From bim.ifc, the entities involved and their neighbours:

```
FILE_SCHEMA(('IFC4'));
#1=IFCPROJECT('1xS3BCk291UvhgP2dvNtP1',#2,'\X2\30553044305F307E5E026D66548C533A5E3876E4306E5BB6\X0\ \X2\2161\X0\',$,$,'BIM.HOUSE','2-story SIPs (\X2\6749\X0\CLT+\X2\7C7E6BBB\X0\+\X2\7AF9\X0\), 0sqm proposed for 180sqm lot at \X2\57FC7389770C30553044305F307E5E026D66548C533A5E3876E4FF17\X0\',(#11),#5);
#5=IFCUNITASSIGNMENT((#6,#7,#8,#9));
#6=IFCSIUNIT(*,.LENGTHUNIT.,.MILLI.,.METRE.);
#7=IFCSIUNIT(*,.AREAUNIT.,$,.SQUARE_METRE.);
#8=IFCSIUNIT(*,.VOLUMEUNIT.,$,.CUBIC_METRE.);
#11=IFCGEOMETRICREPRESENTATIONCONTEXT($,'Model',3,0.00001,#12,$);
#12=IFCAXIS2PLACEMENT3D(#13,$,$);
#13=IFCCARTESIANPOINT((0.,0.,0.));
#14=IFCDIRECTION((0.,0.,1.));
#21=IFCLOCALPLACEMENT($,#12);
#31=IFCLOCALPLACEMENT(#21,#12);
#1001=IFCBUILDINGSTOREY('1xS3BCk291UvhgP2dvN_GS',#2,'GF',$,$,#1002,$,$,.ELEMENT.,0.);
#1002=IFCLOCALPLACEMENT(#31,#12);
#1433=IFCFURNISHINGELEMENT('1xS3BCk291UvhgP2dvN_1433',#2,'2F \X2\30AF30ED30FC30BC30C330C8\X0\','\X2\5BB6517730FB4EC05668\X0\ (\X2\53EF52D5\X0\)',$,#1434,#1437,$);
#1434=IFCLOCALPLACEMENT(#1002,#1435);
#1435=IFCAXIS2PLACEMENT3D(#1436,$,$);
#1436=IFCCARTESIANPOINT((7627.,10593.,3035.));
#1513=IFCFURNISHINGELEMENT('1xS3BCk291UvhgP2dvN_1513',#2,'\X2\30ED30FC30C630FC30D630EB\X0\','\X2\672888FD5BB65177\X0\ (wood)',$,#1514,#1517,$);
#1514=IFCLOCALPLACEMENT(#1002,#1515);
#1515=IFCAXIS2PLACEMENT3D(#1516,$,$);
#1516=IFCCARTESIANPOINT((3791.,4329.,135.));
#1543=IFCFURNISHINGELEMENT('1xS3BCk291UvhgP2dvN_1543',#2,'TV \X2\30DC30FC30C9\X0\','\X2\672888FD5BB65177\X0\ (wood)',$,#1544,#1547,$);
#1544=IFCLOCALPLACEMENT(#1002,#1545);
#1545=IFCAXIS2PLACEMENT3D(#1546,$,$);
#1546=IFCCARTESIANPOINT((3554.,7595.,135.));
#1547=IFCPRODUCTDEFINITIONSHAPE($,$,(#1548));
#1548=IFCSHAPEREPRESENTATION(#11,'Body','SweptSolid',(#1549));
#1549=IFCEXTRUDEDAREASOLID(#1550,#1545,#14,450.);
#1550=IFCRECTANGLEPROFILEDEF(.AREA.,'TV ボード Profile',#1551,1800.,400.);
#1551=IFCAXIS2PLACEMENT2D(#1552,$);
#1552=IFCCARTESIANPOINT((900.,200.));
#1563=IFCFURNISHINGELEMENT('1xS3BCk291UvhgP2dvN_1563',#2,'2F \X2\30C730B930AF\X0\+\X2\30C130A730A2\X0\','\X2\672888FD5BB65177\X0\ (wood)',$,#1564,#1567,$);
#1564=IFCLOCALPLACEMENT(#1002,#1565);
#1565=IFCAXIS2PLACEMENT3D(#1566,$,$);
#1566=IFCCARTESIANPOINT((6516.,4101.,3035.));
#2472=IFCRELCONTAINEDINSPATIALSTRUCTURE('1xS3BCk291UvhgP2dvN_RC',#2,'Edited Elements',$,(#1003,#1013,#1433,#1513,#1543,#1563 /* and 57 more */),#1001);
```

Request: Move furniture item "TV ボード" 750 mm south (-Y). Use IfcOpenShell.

```python
import ifcopenshell
import ifcopenshell.api.geometry
import ifcopenshell.util.placement
import ifcopenshell.util.unit

model = ifcopenshell.open("bim.ifc")
unit_scale = ifcopenshell.util.unit.calculate_unit_scale(model)

item = model.by_id(1543)
matrix = ifcopenshell.util.placement.get_local_placement(item.ObjectPlacement)
matrix[1, 3] -= 0.75 / unit_scale
ifcopenshell.api.geometry.edit_object_placement(model, product=item, matrix=matrix, is_si=False)

print(ifcopenshell.util.placement.get_local_placement(item.ObjectPlacement).round(3) + 0.0)

model.write("bim-out.ifc")
```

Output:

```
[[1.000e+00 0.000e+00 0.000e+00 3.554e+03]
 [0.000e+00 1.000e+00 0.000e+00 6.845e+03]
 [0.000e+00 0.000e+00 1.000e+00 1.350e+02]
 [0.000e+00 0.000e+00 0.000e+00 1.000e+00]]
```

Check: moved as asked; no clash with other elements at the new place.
